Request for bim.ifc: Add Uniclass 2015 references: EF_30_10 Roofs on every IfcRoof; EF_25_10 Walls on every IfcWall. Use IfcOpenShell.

First a look at what the model holds.

```python
import ifcopenshell

model = ifcopenshell.open("bim.ifc")
print(model.schema)
print("classifications:", [c.Name for c in model.by_type("IfcClassification")])
for ifc_class in ("IfcDoor", "IfcRoof", "IfcStair", "IfcWall", "IfcWindow"):
    print(ifc_class, len(model.by_type(ifc_class)))
```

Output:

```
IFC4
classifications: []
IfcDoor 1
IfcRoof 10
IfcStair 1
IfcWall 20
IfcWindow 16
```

```python
import ifcopenshell
import ifcopenshell.api.classification

model = ifcopenshell.open("bim.ifc")

system = ifcopenshell.api.classification.add_classification(model, classification="Uniclass 2015")

codes = {
    "IfcRoof": ("EF_30_10", "Roofs"),
    "IfcWall": ("EF_25_10", "Walls"),
}
for ifc_class, (code, name) in codes.items():
    products = model.by_type(ifc_class)
    ifcopenshell.api.classification.add_reference(
        model, products=products, classification=system, identification=code, name=name
    )
    print(code, len(products))

model.write("bim_v2.ifc")
```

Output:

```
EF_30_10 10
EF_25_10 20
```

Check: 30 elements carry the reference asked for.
